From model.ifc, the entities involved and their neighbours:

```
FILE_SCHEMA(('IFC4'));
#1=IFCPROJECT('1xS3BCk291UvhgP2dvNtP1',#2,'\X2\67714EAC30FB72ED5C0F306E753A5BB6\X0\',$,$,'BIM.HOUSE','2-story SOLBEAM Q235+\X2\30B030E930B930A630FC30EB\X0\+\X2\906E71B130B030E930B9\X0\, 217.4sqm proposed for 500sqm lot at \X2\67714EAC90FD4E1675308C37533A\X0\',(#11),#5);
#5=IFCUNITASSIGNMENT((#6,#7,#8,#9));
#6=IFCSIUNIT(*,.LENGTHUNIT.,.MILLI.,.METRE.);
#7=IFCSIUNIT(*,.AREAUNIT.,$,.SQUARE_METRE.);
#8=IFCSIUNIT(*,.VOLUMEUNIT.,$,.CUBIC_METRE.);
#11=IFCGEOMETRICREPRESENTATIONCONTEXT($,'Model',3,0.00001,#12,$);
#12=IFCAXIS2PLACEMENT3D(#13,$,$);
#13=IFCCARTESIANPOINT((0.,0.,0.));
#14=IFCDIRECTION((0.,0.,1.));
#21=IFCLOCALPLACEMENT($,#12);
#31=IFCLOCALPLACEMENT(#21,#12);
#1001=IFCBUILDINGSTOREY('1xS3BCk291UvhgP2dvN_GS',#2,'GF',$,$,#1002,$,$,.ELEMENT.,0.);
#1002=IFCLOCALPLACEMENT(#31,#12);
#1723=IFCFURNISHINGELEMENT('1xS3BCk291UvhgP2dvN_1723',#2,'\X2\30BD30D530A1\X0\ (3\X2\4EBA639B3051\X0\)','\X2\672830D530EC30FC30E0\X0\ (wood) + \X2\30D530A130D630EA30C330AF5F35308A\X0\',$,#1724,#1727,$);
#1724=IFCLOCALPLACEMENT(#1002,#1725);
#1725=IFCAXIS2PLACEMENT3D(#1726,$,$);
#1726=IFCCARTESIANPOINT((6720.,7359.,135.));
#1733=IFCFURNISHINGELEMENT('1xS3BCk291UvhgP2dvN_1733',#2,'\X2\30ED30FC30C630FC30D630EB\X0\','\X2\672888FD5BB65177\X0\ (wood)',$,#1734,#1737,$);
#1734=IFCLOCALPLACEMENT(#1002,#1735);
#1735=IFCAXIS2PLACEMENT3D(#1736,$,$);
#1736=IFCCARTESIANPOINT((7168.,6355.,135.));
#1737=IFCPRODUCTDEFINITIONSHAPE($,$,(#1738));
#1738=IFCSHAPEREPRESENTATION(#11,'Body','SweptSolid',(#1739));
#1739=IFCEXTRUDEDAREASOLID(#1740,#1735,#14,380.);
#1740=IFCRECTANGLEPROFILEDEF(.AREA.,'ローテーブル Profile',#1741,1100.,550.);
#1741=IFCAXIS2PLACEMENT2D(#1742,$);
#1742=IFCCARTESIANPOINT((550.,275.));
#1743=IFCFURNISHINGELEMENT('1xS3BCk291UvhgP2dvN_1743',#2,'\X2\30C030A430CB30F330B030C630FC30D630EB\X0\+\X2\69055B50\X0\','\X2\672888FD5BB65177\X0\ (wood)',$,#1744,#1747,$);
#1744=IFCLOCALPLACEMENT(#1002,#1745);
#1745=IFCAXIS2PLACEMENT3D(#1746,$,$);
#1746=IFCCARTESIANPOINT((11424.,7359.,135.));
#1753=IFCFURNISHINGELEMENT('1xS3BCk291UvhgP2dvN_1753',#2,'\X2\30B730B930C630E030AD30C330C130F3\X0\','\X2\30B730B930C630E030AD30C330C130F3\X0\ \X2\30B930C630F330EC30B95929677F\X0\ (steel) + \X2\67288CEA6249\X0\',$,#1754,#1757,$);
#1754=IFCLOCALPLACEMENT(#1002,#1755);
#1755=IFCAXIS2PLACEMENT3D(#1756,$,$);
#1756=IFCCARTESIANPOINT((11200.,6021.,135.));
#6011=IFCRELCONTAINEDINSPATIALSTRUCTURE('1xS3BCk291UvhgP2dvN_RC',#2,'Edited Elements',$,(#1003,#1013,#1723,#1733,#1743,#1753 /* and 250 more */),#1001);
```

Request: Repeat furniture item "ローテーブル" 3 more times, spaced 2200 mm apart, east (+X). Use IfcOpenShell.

```python
import numpy as np
import ifcopenshell
import ifcopenshell.api.geometry
import ifcopenshell.api.root
import ifcopenshell.util.element
import ifcopenshell.util.placement

model = ifcopenshell.open("model.ifc")


def reuse_history(source, copy):
    """copy_class also copies each property set's owner history, people and application; keep the originals."""
    for rel in copy.IsDefinedBy:
        if rel.is_a("IfcRelDefinesByProperties") and (history := rel.RelatingPropertyDefinition.OwnerHistory):
            rel.RelatingPropertyDefinition.OwnerHistory = source.OwnerHistory
            ifcopenshell.util.element.remove_deep2(model, history)


source = model.by_guid("1xS3BCk291UvhgP2dvN_1733")
base = ifcopenshell.util.placement.get_local_placement(source.ObjectPlacement)
step = np.array([1.0, 0.0, 0.0]) * 2200.0

for i in range(1, 4):
    copy = ifcopenshell.api.root.copy_class(model, product=source)
    copy.Representation = ifcopenshell.util.element.copy_deep(
        model, source.Representation, exclude=["IfcGeometricRepresentationContext", "IfcRepresentationMap"]
    )
    reuse_history(source, copy)
    matrix = base.copy()
    matrix[:3, 3] += i * step
    print("added at", matrix[:3, 3].round(3) + 0.0)
    ifcopenshell.api.geometry.edit_object_placement(model, product=copy, matrix=matrix, is_si=False)

model.write("model-out.ifc")
```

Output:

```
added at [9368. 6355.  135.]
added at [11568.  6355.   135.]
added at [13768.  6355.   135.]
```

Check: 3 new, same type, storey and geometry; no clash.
